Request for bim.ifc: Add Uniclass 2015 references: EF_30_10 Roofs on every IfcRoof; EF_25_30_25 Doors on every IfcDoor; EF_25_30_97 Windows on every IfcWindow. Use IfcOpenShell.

First a look at what the model holds.

```python
import ifcopenshell

model = ifcopenshell.open("bim.ifc")
print(model.schema)
print("classifications:", [c.Name for c in model.by_type("IfcClassification")])
for ifc_class in ("IfcDoor", "IfcRoof", "IfcStair", "IfcWall", "IfcWindow"):
    print(ifc_class, len(model.by_type(ifc_class)))
```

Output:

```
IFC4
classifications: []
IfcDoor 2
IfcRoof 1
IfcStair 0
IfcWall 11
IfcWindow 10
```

```python
import ifcopenshell
import ifcopenshell.api.classification

model = ifcopenshell.open("bim.ifc")

system = ifcopenshell.api.classification.add_classification(model, classification="Uniclass 2015")

codes = {
    "IfcRoof": ("EF_30_10", "Roofs"),
    "IfcDoor": ("EF_25_30_25", "Doors"),
    "IfcWindow": ("EF_25_30_97", "Windows"),
}
for ifc_class, (code, name) in codes.items():
    products = model.by_type(ifc_class)
    ifcopenshell.api.classification.add_reference(
        model, products=products, classification=system, identification=code, name=name
    )
    print(code, len(products))

model.write("bim_updated.ifc")
```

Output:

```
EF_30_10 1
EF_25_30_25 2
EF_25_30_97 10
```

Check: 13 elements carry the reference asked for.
